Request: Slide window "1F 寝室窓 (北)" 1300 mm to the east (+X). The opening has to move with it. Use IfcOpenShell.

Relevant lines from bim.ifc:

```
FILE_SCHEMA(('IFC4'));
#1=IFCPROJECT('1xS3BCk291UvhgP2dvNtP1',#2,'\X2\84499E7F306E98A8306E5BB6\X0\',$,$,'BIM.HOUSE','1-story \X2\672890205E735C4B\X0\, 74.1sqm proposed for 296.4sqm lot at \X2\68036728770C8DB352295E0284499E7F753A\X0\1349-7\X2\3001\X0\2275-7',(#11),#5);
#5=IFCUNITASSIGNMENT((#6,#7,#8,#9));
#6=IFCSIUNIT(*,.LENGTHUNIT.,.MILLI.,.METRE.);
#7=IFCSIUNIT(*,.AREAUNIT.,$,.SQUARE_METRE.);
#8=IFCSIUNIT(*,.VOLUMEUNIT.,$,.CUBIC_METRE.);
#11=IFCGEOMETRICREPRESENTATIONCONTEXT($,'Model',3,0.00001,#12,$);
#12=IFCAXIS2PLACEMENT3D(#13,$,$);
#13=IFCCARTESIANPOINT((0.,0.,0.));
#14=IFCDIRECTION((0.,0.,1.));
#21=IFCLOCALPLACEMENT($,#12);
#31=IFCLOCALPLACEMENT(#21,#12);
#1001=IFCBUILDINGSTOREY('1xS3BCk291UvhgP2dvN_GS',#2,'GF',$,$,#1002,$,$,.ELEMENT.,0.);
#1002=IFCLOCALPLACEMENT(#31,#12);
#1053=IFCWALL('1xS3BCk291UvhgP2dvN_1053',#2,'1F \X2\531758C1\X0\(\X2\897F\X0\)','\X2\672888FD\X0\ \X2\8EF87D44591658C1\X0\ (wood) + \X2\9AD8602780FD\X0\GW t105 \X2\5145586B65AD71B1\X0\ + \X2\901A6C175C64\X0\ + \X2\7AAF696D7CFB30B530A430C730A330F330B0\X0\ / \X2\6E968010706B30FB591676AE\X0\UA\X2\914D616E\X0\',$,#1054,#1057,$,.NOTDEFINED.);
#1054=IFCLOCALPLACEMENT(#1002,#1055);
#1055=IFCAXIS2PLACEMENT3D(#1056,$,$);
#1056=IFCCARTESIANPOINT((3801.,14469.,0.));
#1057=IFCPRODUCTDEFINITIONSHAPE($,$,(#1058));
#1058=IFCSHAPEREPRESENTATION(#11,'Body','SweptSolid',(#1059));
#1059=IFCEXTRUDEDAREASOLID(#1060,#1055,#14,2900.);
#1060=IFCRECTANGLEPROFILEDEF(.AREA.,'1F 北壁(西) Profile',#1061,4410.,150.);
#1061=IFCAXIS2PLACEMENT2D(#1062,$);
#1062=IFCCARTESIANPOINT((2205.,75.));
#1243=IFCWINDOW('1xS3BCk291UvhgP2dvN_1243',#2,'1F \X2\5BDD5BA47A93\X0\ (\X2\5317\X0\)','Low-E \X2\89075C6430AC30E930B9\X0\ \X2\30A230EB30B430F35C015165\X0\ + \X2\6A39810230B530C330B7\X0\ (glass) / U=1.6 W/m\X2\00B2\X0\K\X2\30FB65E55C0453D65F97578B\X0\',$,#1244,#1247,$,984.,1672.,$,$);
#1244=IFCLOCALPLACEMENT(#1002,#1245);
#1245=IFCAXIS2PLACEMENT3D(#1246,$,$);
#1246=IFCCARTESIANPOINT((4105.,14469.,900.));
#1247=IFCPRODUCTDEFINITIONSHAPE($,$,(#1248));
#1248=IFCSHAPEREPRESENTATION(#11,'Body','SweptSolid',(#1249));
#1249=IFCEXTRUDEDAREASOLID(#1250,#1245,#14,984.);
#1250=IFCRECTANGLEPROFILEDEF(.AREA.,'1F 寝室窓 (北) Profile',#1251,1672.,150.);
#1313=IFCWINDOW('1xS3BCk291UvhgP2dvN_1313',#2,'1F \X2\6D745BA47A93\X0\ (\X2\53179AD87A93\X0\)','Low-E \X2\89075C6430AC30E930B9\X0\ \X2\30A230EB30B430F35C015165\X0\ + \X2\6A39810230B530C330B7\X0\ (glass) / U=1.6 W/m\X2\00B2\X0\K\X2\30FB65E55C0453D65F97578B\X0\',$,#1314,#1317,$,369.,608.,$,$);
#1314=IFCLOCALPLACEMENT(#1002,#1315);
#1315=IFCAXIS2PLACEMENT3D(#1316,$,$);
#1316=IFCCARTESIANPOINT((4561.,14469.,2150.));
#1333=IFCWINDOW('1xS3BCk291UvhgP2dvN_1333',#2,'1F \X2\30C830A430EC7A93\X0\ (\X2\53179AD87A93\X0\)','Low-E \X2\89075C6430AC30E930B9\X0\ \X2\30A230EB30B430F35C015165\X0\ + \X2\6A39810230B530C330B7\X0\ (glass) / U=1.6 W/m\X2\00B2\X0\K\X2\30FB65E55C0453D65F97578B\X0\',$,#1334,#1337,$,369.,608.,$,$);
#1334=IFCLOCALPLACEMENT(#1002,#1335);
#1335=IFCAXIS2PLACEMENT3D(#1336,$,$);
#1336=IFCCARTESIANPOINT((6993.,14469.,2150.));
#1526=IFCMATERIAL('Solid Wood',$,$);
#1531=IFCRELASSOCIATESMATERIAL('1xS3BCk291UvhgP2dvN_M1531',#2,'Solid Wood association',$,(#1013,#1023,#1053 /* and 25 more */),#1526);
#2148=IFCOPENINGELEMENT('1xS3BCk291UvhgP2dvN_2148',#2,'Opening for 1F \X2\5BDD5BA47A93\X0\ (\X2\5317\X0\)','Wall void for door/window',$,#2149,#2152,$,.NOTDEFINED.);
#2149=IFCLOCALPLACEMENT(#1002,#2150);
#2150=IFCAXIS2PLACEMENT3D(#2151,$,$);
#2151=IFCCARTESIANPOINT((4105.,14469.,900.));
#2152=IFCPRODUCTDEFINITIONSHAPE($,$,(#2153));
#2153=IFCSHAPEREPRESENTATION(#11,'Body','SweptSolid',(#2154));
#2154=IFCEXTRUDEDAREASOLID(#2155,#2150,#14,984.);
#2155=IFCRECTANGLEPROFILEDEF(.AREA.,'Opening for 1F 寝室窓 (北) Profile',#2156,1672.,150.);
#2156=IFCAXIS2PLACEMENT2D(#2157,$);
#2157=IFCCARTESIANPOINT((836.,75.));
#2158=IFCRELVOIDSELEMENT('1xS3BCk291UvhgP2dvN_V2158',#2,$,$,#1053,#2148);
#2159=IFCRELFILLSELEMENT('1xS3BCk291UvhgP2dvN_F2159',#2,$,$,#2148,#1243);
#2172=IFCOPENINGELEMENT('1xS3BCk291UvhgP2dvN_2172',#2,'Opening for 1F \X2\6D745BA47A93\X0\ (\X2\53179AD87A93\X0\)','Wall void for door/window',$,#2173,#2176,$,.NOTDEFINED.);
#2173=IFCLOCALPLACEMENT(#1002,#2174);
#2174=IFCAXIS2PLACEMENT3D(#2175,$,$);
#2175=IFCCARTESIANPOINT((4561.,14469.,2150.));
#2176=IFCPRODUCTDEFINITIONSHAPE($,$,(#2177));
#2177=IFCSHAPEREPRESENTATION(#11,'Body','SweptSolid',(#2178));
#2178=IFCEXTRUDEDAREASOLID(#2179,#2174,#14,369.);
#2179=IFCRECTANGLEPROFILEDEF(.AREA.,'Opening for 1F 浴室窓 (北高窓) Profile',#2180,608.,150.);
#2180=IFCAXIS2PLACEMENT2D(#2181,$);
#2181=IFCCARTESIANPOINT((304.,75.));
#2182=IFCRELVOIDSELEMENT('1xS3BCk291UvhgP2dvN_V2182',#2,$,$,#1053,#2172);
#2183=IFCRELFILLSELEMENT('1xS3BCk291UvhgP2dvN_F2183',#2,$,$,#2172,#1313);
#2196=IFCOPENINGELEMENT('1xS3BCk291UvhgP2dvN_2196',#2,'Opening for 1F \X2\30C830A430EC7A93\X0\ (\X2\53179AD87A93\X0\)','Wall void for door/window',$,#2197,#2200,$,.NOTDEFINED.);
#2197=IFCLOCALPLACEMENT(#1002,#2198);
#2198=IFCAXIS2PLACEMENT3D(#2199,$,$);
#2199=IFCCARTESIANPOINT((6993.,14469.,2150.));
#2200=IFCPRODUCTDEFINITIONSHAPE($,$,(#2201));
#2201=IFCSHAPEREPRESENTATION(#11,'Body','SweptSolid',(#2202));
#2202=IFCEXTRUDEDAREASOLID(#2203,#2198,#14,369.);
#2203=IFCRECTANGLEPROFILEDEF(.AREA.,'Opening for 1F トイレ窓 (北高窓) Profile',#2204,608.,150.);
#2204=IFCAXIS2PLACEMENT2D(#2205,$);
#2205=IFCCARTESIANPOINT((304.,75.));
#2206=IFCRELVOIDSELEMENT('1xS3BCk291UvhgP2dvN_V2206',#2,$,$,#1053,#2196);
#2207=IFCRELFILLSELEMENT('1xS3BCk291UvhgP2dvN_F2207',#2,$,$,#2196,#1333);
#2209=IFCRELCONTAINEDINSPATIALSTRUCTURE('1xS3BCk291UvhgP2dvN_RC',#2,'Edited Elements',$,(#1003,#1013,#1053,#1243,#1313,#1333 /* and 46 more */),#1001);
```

```python
import ifcopenshell
import ifcopenshell.api.geometry
import ifcopenshell.util.placement
import ifcopenshell.util.unit

model = ifcopenshell.open("bim.ifc")
unit_scale = ifcopenshell.util.unit.calculate_unit_scale(model)

window = model.by_id(1243)
opening = window.FillsVoids[0].RelatingOpeningElement
wall = opening.VoidsElements[0].RelatingBuildingElement

wall_matrix = ifcopenshell.util.placement.get_local_placement(wall.ObjectPlacement)
shift = wall_matrix[:3, 0] * 1.3 / unit_scale
before = ifcopenshell.util.placement.get_local_placement(window.ObjectPlacement)[:3, 3].copy()

# The window is not placed relative to its opening, so move both.
for product in (opening, window):
    matrix = ifcopenshell.util.placement.get_local_placement(product.ObjectPlacement)
    matrix[:3, 3] += shift
    ifcopenshell.api.geometry.edit_object_placement(model, product=product, matrix=matrix, is_si=False)

after = ifcopenshell.util.placement.get_local_placement(window.ObjectPlacement)[:3, 3]
print("window moved by", (after - before).round(3) + 0.0)

model.write("bim_updated.ifc")
```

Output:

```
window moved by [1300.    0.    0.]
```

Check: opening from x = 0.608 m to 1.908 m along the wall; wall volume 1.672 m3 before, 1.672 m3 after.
